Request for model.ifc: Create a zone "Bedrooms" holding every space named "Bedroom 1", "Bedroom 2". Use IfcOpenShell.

First a look at what the model holds.

```python
import ifcopenshell

model = ifcopenshell.open("model.ifc")
print(model.schema)
seen = {}
for space in model.by_type("IfcSpace"):
    seen[space.LongName] = seen.get(space.LongName, 0) + 1
for name, count in sorted(seen.items(), key=str):
    print(count, "x", name)
print("zones:", [z.Name for z in model.by_type("IfcZone")][:20])
```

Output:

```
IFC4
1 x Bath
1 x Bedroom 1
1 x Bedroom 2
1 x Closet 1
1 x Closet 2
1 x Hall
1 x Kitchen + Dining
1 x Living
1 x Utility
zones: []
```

```python
import ifcopenshell
import ifcopenshell.api.group
import ifcopenshell.api.root

model = ifcopenshell.open("model.ifc")

names = {"Bedroom 1", "Bedroom 2"}
spaces = [s for s in model.by_type("IfcSpace") if s.LongName in names]

zone = ifcopenshell.api.root.create_entity(model, ifc_class="IfcZone", name="Bedrooms")
ifcopenshell.api.group.assign_group(model, products=spaces, group=zone)
print(len(spaces), "spaces in", zone.Name)

model.write("model_updated.ifc")
```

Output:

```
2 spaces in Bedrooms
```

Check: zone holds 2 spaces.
